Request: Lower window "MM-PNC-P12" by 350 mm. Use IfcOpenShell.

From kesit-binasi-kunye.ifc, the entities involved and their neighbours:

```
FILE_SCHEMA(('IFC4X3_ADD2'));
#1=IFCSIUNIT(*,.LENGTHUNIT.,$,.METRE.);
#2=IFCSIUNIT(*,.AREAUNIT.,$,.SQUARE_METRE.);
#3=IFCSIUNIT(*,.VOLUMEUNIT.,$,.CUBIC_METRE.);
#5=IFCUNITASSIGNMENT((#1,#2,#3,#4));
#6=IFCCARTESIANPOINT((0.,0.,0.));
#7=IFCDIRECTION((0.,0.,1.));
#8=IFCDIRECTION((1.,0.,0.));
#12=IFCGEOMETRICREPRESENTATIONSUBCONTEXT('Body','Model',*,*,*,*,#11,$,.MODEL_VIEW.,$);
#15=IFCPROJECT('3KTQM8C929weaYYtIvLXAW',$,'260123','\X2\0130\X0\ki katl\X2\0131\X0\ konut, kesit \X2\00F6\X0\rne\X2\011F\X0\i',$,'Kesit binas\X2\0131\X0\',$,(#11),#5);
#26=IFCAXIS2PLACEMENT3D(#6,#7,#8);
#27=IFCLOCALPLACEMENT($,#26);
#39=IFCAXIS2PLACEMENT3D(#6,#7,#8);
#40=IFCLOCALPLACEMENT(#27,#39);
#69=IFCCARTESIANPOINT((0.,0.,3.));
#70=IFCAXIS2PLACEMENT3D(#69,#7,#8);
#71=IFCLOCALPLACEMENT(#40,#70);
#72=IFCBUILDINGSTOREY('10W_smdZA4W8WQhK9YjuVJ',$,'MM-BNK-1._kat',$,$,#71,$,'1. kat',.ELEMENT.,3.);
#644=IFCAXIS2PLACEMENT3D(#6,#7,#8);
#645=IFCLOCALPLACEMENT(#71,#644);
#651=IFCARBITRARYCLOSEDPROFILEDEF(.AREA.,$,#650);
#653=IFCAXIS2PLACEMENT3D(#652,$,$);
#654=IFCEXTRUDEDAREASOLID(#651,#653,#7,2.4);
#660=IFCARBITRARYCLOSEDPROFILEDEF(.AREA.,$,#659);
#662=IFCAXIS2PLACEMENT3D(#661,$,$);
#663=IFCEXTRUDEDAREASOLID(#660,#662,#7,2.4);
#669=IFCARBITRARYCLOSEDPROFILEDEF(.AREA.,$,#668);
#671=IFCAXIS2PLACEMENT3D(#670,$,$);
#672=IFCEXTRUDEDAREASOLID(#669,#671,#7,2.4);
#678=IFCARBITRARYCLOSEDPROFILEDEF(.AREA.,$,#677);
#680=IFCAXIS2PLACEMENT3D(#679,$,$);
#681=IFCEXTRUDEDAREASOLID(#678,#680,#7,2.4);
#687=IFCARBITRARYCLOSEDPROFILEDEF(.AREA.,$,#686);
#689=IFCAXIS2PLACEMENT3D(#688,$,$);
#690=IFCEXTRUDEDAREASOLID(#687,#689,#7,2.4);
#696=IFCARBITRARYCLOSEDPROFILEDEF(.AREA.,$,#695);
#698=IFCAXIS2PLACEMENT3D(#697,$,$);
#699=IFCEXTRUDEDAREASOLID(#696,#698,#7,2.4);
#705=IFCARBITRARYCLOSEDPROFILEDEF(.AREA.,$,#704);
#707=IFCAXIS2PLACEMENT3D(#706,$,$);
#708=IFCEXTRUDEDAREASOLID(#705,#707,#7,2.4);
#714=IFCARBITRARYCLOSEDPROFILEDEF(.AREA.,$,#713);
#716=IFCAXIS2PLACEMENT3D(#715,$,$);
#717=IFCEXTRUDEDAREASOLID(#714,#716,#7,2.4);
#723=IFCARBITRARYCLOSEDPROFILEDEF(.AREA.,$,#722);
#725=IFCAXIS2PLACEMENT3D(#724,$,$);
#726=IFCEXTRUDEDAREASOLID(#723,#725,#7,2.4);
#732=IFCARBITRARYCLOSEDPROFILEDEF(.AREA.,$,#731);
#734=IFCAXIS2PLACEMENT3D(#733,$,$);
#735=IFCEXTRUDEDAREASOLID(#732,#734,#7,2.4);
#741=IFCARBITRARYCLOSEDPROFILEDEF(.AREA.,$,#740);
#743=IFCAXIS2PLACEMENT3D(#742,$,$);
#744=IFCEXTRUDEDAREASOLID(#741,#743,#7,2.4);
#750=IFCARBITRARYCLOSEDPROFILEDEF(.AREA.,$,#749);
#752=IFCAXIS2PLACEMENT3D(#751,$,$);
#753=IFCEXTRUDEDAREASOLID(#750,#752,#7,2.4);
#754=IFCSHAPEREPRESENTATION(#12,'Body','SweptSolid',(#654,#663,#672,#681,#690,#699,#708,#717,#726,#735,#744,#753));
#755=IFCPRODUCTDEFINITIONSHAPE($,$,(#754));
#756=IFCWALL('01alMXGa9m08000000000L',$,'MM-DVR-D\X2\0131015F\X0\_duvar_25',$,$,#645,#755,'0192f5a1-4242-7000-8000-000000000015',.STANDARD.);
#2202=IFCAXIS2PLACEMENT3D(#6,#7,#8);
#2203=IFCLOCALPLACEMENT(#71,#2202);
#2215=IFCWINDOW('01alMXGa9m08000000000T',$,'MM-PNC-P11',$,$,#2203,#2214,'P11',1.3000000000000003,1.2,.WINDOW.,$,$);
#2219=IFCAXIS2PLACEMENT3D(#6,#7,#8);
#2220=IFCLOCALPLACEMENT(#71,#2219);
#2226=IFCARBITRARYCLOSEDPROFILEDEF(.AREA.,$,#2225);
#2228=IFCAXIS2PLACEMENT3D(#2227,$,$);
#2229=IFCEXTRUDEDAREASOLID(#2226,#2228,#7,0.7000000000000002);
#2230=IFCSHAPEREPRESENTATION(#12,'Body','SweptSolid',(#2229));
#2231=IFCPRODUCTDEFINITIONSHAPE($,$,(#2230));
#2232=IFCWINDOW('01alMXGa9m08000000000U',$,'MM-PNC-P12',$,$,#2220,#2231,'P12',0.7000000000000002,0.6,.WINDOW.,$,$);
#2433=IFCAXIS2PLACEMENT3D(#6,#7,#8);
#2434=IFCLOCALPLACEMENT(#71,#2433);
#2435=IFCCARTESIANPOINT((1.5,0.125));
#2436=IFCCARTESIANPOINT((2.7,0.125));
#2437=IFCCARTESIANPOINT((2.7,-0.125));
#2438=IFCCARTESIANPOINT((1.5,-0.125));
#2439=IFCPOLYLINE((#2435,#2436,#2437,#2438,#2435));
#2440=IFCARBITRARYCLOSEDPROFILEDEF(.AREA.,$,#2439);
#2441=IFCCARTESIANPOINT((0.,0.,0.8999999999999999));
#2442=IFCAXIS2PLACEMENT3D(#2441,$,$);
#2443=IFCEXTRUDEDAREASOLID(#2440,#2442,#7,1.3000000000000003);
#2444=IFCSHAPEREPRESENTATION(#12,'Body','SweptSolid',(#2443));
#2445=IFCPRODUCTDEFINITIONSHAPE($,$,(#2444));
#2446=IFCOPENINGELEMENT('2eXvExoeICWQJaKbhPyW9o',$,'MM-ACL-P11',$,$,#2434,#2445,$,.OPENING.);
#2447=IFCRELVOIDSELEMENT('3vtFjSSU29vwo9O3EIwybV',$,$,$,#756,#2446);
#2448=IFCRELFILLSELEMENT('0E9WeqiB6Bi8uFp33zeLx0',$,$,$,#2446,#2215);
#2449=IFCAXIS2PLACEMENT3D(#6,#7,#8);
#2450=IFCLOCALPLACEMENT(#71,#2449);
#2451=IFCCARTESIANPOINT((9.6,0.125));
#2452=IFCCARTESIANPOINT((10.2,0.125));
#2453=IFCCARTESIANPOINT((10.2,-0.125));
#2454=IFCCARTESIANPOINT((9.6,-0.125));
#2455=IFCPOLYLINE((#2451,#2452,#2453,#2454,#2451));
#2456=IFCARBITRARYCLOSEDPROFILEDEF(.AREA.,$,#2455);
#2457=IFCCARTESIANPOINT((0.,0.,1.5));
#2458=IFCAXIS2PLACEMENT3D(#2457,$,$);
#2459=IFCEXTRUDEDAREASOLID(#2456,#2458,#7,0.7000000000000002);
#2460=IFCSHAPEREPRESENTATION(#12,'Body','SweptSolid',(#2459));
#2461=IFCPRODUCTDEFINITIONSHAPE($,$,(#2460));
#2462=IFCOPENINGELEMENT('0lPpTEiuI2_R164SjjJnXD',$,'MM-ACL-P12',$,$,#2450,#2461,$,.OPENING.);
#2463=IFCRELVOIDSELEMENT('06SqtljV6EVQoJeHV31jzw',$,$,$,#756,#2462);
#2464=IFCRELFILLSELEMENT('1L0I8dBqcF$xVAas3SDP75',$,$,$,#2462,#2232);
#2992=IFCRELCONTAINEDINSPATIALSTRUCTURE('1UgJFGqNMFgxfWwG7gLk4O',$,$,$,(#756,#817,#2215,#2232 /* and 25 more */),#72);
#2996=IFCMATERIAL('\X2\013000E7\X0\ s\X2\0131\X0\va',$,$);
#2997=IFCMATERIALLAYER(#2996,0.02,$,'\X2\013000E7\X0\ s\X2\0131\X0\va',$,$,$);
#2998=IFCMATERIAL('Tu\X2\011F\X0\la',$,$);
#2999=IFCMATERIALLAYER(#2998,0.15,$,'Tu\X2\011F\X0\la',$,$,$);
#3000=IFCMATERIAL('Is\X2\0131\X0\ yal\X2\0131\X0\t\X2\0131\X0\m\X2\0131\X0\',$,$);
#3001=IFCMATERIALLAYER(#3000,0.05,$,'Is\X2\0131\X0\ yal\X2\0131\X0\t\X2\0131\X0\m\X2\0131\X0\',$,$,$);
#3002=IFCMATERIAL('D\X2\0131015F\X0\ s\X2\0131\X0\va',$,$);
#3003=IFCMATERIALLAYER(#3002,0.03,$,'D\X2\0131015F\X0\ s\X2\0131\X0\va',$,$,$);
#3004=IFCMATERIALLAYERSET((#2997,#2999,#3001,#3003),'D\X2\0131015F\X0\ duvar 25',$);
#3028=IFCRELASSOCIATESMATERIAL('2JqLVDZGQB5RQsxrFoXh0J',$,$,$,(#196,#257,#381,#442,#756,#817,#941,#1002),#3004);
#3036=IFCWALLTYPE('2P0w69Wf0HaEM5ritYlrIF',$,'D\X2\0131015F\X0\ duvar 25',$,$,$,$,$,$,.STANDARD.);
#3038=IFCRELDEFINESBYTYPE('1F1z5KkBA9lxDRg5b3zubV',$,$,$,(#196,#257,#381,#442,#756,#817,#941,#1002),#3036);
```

```python
import numpy as np
import ifcopenshell
import ifcopenshell.api.geometry
import ifcopenshell.util.placement
import ifcopenshell.util.unit

model = ifcopenshell.open("kesit-binasi-kunye.ifc")
unit_scale = ifcopenshell.util.unit.calculate_unit_scale(model)

window = model.by_guid("01alMXGa9m08000000000U")
opening = window.FillsVoids[0].RelatingOpeningElement
dz = -0.35

shift = np.array([0.0, 0.0, dz])
# The window is not placed relative to its opening, so move both.
for product in (opening, window):
    matrix = ifcopenshell.util.placement.get_local_placement(product.ObjectPlacement)
    matrix[:3, 3] += shift
    ifcopenshell.api.geometry.edit_object_placement(model, product=product, matrix=matrix, is_si=False)

print(f"moved by {dz * unit_scale:+.3f} m")

model.write("kesit-binasi-kunye-out.ifc")
```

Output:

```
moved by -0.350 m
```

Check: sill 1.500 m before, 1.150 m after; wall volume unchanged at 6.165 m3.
